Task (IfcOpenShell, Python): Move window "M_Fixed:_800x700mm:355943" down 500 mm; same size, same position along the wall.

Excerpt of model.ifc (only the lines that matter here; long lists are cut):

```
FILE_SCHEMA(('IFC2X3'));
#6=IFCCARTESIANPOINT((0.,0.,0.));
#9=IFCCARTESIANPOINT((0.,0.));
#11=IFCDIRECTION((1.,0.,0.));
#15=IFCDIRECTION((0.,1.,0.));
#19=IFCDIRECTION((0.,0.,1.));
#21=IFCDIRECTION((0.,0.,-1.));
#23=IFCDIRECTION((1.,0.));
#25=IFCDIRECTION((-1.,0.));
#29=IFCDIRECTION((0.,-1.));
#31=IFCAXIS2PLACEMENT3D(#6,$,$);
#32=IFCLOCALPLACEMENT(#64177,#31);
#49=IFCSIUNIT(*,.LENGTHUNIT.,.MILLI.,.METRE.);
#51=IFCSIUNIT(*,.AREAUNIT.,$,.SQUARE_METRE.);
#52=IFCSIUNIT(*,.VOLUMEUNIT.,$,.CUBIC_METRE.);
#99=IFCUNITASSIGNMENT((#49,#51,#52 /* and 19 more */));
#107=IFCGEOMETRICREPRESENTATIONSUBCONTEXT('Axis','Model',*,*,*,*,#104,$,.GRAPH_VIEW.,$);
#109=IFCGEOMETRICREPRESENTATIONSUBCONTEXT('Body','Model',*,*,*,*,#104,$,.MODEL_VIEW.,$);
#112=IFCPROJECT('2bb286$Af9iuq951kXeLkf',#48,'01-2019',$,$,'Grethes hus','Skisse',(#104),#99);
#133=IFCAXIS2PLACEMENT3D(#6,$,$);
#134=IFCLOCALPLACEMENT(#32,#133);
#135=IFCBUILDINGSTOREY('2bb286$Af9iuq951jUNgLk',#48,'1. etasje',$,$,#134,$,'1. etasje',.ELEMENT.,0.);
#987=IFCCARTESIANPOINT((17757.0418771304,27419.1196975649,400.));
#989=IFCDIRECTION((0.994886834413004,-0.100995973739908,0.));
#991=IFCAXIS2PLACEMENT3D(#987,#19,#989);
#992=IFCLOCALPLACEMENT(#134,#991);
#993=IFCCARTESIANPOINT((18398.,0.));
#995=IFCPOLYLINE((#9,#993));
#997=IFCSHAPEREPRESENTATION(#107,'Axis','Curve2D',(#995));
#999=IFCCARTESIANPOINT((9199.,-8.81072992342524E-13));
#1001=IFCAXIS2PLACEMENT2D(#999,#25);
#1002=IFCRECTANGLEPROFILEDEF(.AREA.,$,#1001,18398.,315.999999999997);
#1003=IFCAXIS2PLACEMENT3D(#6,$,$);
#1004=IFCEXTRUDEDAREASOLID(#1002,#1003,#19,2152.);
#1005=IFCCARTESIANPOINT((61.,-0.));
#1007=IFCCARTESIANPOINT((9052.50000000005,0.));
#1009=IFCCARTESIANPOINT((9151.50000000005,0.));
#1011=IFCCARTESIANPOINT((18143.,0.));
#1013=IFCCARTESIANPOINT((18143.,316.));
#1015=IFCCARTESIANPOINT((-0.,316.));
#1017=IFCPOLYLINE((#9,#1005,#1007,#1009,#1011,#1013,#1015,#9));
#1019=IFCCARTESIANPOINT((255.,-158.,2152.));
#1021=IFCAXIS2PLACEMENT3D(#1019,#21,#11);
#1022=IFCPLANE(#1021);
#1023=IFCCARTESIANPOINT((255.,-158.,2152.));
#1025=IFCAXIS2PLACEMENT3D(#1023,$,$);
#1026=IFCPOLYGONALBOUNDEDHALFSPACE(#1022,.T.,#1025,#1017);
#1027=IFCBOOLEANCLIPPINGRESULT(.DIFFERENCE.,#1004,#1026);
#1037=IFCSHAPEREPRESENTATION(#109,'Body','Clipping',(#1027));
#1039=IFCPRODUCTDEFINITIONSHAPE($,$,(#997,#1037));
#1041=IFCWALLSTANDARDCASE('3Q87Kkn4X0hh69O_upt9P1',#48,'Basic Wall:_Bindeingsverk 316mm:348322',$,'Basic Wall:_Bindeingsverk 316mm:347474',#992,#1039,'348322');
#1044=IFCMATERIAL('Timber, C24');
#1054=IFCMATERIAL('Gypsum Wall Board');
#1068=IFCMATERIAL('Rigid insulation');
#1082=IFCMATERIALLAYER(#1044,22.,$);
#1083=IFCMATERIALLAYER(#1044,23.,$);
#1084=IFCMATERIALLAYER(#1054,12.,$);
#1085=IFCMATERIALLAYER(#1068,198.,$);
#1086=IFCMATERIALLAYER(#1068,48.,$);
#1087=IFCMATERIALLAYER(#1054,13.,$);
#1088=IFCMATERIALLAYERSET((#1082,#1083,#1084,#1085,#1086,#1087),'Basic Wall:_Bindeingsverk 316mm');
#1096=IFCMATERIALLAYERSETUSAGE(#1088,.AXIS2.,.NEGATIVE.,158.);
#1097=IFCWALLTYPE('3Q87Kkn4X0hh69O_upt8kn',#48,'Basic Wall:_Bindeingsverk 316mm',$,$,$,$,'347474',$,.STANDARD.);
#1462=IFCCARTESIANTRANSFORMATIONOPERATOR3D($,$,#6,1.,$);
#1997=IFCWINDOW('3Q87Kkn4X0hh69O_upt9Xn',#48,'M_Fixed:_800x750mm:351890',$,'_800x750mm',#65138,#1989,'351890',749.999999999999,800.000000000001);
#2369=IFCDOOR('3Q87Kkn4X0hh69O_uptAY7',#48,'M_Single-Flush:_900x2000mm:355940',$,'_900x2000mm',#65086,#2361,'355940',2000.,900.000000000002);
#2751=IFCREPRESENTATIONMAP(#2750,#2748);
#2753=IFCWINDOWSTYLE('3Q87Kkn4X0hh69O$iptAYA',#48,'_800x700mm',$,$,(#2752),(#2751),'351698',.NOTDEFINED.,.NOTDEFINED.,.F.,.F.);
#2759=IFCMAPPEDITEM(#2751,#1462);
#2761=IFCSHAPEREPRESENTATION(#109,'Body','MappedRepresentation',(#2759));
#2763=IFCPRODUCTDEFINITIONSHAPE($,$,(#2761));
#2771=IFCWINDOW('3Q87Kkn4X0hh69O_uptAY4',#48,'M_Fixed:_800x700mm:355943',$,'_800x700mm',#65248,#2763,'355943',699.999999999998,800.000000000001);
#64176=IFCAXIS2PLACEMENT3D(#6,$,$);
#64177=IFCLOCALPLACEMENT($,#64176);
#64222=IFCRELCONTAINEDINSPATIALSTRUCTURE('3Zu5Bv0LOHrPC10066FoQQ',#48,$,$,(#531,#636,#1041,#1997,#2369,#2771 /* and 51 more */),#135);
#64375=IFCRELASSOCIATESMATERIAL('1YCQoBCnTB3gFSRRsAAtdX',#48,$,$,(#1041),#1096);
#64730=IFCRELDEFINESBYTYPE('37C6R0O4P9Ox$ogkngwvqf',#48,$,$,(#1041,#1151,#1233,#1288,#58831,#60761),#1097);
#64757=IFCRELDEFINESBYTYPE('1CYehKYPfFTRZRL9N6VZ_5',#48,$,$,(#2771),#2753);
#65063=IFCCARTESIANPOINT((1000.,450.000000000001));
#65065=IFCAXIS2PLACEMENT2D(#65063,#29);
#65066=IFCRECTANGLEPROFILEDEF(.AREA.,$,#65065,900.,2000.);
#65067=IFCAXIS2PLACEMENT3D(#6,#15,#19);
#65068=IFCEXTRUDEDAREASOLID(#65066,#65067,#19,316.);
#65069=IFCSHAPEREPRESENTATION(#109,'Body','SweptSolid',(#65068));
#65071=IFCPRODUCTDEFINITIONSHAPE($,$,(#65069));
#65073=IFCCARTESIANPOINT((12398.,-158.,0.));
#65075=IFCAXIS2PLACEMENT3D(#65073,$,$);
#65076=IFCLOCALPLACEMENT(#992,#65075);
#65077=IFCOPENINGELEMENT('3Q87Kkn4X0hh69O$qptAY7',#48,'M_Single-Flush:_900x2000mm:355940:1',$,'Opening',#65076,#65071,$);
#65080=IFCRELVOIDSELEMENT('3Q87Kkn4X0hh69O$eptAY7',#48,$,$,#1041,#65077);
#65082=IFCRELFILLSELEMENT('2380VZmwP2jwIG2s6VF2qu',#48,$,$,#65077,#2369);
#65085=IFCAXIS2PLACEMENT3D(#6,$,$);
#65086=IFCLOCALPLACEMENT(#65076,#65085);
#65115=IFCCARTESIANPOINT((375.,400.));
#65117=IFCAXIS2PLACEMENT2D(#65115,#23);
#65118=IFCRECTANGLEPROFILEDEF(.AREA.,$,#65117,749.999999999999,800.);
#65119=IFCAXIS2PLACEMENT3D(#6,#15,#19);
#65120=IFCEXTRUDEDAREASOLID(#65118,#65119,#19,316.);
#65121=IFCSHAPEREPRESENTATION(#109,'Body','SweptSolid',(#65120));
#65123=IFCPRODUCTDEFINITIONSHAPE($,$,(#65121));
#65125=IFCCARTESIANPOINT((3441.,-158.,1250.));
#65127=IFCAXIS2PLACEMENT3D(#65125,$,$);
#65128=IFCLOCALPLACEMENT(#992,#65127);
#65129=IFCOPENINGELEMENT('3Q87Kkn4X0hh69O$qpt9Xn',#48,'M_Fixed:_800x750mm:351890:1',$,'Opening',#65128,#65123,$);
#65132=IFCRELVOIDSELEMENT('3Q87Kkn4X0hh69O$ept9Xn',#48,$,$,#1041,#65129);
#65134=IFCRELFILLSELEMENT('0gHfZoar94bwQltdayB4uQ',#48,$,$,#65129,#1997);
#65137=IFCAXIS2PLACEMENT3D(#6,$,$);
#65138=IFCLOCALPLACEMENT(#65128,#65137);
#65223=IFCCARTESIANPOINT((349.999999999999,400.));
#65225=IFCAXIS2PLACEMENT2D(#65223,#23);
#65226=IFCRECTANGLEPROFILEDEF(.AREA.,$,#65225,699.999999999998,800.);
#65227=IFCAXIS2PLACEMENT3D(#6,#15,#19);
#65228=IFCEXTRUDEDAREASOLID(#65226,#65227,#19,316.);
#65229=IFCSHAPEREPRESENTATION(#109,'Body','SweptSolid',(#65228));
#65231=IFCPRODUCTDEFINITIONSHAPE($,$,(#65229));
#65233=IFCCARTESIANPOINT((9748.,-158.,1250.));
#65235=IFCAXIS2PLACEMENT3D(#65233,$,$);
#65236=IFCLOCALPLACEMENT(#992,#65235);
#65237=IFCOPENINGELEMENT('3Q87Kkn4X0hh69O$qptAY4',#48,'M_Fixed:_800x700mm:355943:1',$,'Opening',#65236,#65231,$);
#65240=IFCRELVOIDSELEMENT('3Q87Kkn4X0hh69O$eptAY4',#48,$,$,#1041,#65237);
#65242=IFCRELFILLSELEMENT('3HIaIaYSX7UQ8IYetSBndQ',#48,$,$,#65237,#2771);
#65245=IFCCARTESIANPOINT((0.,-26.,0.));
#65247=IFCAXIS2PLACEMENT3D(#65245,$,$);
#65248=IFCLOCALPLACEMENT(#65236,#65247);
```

```python
import numpy as np
import ifcopenshell
import ifcopenshell.api.geometry
import ifcopenshell.util.placement
import ifcopenshell.util.unit

model = ifcopenshell.open("model.ifc")
unit_scale = ifcopenshell.util.unit.calculate_unit_scale(model)

window = model.by_guid("3Q87Kkn4X0hh69O_uptAY4")
opening = window.FillsVoids[0].RelatingOpeningElement
dz = -0.5 / unit_scale

shift = np.array([0.0, 0.0, dz])
# The window is placed relative to its opening, so it follows when the opening moves.
matrix = ifcopenshell.util.placement.get_local_placement(opening.ObjectPlacement)
matrix[:3, 3] += shift
ifcopenshell.api.geometry.edit_object_placement(
    model, product=opening, matrix=matrix, is_si=False, should_transform_children=True
)

print(f"moved by {dz * unit_scale:+.3f} m")

model.write("model-out.ifc")
```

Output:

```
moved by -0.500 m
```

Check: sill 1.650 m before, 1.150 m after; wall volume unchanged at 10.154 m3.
